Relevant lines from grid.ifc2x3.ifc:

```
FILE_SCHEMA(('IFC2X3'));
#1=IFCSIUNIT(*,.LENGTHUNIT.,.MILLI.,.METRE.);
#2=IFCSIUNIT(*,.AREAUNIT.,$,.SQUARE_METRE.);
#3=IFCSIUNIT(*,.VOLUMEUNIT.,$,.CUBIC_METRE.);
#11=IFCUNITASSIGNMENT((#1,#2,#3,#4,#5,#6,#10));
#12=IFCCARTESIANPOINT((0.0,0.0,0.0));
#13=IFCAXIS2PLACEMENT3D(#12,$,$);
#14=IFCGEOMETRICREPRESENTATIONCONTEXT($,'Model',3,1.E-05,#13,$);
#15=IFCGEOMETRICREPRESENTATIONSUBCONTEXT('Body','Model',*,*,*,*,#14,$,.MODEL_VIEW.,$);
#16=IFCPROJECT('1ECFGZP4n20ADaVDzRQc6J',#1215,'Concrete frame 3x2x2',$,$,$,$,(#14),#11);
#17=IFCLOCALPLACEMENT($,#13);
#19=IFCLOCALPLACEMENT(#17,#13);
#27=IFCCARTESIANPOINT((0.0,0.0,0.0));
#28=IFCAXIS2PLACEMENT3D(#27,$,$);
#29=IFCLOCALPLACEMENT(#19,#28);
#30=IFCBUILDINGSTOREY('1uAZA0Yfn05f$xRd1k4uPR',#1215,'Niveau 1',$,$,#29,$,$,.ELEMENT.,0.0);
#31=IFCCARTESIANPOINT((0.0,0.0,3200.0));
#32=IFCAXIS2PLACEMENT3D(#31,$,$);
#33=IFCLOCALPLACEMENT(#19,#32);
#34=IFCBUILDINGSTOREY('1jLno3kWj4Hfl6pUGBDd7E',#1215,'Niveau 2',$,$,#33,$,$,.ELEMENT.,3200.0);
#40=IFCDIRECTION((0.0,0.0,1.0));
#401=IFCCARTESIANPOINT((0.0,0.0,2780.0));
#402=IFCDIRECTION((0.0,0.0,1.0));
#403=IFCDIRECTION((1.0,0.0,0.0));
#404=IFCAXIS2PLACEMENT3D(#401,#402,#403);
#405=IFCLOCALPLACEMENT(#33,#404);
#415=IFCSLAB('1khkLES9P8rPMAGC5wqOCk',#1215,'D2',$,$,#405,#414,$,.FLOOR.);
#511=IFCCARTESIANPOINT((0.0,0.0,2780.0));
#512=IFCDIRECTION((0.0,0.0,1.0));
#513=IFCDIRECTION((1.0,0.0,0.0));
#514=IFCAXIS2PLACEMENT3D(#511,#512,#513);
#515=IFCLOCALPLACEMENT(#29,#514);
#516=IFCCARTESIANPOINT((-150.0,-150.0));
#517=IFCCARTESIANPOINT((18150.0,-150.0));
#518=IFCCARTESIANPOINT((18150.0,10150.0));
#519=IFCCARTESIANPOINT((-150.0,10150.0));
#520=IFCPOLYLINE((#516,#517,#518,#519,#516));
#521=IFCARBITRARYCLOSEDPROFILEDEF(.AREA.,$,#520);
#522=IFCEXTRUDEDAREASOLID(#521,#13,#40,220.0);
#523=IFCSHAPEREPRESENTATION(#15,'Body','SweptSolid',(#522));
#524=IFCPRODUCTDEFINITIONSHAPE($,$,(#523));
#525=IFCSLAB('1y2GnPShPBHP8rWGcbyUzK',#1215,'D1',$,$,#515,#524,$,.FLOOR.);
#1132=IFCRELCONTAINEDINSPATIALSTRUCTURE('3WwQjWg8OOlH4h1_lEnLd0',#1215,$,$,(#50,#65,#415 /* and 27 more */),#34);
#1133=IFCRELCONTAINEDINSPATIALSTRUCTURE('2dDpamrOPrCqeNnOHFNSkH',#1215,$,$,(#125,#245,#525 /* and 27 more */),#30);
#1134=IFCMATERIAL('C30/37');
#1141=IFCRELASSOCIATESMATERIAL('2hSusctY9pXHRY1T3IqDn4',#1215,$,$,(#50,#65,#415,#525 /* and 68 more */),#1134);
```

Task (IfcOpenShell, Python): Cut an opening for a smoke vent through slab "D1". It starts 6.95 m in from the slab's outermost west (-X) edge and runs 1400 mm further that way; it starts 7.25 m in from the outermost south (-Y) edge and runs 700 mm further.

```python
import numpy as np
import ifcopenshell
import ifcopenshell.api.feature
import ifcopenshell.api.geometry
import ifcopenshell.api.root
import ifcopenshell.geom
import ifcopenshell.util.placement
import ifcopenshell.util.representation
import ifcopenshell.util.shape
import ifcopenshell.util.unit

model = ifcopenshell.open("grid.ifc2x3.ifc")
unit_scale = ifcopenshell.util.unit.calculate_unit_scale(model)
settings = ifcopenshell.geom.settings()


def volume(element):
    """Net volume in cubic metres, openings subtracted."""
    shape = ifcopenshell.geom.create_shape(settings, element)
    return ifcopenshell.util.shape.get_volume(shape.geometry)


slab = model.by_guid("1y2GnPShPBHP8rWGcbyUzK")
before = volume(slab)

# Extent in the slab's own axes, in metres. The edges named are its -X and -Y sides.
slab_shape = ifcopenshell.geom.create_shape(settings, slab)
vertices = ifcopenshell.util.shape.get_vertices(slab_shape.geometry)
x_min, y_min, bottom = vertices.min(axis=0)
top = vertices[:, 2].max()

opening = ifcopenshell.api.root.create_entity(model, ifc_class="IfcOpeningElement", name="Smoke vent opening")
context = ifcopenshell.util.representation.get_context(model, "Model", "Body", "MODEL_VIEW")
width, depth = 1.4, 0.7
outline = [(0.0, 0.0), (width, 0.0), (width, depth), (0.0, depth), (0.0, 0.0)]
# Overshoot both faces by 50 mm so the cut is clean.
shape = ifcopenshell.api.geometry.add_slab_representation(
    model, context=context, depth=top - bottom + 0.1, polyline=outline
)
ifcopenshell.api.geometry.assign_representation(model, product=opening, representation=shape)

matrix = ifcopenshell.util.placement.get_local_placement(slab.ObjectPlacement)
matrix[:, 3] = matrix @ np.append(np.array([x_min + 6.95, y_min + 7.25, bottom - 0.05]) / unit_scale, 1.0)
ifcopenshell.api.geometry.edit_object_placement(model, product=opening, matrix=matrix, is_si=False)
ifcopenshell.api.feature.add_feature(model, feature=opening, element=slab)

after = volume(slab)

print(f"slab volume {before:.3f} -> {after:.3f} m3")

model.write("grid.ifc2x3_v2.ifc")
```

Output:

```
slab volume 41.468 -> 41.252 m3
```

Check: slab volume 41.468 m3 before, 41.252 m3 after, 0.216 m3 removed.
